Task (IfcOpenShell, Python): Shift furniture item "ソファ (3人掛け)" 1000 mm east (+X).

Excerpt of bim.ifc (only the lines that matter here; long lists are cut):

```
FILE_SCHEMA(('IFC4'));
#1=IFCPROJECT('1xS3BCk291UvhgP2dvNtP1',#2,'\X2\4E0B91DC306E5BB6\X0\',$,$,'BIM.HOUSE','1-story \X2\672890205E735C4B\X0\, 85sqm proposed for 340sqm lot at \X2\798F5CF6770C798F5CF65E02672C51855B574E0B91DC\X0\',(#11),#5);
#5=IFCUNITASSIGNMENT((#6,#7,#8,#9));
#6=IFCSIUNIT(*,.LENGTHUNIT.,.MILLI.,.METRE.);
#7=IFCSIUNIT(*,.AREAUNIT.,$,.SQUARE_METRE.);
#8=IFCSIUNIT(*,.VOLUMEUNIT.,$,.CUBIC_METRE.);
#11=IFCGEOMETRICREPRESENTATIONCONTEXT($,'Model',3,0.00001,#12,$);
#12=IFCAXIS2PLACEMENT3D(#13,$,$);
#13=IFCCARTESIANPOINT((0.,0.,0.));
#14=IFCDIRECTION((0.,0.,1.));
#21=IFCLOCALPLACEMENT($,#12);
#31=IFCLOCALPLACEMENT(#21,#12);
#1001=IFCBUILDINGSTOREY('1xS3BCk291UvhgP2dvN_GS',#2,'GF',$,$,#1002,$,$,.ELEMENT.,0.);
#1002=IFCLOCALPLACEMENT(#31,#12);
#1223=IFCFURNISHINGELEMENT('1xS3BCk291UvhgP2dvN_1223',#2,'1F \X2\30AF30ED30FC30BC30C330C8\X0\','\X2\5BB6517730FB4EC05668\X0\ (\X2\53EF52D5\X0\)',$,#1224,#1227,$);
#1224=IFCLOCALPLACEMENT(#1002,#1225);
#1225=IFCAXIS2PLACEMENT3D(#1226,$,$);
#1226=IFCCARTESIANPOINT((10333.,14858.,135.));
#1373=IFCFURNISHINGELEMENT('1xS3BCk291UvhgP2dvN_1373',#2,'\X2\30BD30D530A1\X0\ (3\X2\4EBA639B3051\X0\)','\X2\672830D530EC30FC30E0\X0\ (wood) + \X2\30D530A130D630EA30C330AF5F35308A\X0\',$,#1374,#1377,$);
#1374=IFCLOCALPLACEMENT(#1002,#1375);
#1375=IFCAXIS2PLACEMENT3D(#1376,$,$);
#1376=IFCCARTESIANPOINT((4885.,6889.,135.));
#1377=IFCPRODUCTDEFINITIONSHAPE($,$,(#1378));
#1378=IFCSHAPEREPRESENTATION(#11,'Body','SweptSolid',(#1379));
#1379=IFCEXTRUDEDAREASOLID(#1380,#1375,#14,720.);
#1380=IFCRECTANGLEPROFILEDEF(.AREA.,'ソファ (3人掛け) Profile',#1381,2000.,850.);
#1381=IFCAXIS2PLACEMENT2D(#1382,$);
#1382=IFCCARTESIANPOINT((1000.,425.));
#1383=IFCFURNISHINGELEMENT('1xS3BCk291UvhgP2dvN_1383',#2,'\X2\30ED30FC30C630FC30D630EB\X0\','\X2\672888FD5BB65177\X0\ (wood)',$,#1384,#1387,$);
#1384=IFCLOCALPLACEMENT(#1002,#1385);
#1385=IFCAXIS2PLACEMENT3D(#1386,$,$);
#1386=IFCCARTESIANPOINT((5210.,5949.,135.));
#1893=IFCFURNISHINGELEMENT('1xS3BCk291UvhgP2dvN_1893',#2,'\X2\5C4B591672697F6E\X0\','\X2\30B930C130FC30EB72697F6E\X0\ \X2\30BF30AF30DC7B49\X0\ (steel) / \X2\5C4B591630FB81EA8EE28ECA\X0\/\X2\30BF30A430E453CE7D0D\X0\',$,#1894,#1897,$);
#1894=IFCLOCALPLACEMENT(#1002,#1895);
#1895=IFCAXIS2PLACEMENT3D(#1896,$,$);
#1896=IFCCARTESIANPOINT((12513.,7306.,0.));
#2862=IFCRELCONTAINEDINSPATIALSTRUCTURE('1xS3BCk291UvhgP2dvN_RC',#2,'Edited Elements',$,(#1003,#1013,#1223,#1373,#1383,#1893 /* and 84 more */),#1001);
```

```python
import ifcopenshell
import ifcopenshell.api.geometry
import ifcopenshell.util.placement
import ifcopenshell.util.unit

model = ifcopenshell.open("bim.ifc")
unit_scale = ifcopenshell.util.unit.calculate_unit_scale(model)

item = model.by_guid("1xS3BCk291UvhgP2dvN_1373")
matrix = ifcopenshell.util.placement.get_local_placement(item.ObjectPlacement)
matrix[0, 3] += 1 / unit_scale
ifcopenshell.api.geometry.edit_object_placement(model, product=item, matrix=matrix, is_si=False)

print(ifcopenshell.util.placement.get_local_placement(item.ObjectPlacement).round(3) + 0.0)

model.write("bim-out.ifc")
```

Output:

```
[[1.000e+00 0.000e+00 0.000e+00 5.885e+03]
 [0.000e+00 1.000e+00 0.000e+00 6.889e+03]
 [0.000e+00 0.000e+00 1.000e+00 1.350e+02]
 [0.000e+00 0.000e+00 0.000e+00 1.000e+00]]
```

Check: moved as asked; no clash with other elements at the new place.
